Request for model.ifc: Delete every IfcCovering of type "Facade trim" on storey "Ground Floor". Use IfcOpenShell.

First a look at what the model holds.

```python
import ifcopenshell
import ifcopenshell.util.element

model = ifcopenshell.open("model.ifc")
print(model.schema)
storey = next(s for s in model.by_type("IfcBuildingStorey") if s.Name == "Ground Floor")
coverings = [e for e in ifcopenshell.util.element.get_decomposition(storey) if e.is_a("IfcCovering")]
seen = {}
for e in coverings:
    element_type = ifcopenshell.util.element.get_type(e)
    name = element_type.Name if element_type not in (None, e) else None
    seen[name] = seen.get(name, 0) + 1
for name, count in sorted(seen.items(), key=str):
    print(count, "x", name)
```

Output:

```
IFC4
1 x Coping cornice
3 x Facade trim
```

```python
import ifcopenshell
import ifcopenshell.api.root
import ifcopenshell.util.element

model = ifcopenshell.open("model.ifc")

storey = next(s for s in model.by_type("IfcBuildingStorey") if s.Name == "Ground Floor")
coverings = [e for e in ifcopenshell.util.element.get_decomposition(storey) if e.is_a("IfcCovering")]
targets = [e for e in coverings if (t := ifcopenshell.util.element.get_type(e)) not in (None, e) and t.Name == "Facade trim"]

for e in targets:
    ifcopenshell.api.root.remove_product(model, product=e)
print(len(targets), "removed")

model.write("model_updated.ifc")
```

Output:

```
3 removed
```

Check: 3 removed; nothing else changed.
